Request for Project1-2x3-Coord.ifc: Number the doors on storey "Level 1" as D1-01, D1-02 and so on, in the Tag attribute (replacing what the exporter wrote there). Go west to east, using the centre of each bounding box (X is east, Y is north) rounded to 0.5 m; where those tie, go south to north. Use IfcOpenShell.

First a look at what the model holds.

```python
import ifcopenshell
import ifcopenshell.util.element
import ifcopenshell.util.placement

model = ifcopenshell.open("Project1-2x3-Coord.ifc")
print(model.schema)
storey = next(s for s in model.by_type("IfcBuildingStorey") if s.Name == "Level 1")
doors = [e for e in ifcopenshell.util.element.get_decomposition(storey) if e.is_a("IfcDoor")]
for e in sorted(doors, key=lambda e: e.id()):
    origin = ifcopenshell.util.placement.get_local_placement(e.ObjectPlacement)[:3, 3]
    print(e.id(), e.Tag, e.Name, origin.round(2) + 0.0, sep=" | ")
```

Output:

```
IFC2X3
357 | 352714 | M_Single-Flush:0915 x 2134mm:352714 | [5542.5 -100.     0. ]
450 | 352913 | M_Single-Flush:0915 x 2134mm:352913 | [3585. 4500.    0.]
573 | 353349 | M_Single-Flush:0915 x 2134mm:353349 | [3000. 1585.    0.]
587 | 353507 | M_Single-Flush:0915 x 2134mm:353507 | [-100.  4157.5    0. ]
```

```python
import ifcopenshell
import ifcopenshell.geom
import ifcopenshell.util.element
import ifcopenshell.util.shape

model = ifcopenshell.open("Project1-2x3-Coord.ifc")
settings = ifcopenshell.geom.settings()
settings.set("use-world-coords", True)


def centre(element):
    shape = ifcopenshell.geom.create_shape(settings, element)
    return ifcopenshell.util.shape.get_bbox_centroid(shape.geometry)


storey = next(s for s in model.by_type("IfcBuildingStorey") if s.Name == "Level 1")
doors = [e for e in ifcopenshell.util.element.get_decomposition(storey) if e.is_a("IfcDoor")]

# Insertion points can sit at a corner or the storey origin, so sort by the geometry (in metres).
centres = {e: centre(e) for e in doors}
doors.sort(key=lambda e: (round(centres[e][0] / 0.5), centres[e][1]))

for i, e in enumerate(doors, start=1):
    number = f"D1-{i:02d}"
    e.Tag = number
    print(e.id(), number)

model.write("Project1-2x3-Coord_updated.ifc")
```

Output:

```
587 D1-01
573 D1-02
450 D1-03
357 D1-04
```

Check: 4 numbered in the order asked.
